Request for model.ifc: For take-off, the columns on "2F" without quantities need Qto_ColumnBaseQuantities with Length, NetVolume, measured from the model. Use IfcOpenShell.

First a look at what the model holds.

```python
import ifcopenshell
import ifcopenshell.util.element
import ifcopenshell.util.unit

model = ifcopenshell.open("model.ifc")
print(model.schema)
for unit_type in ("LENGTHUNIT", "AREAUNIT", "VOLUMEUNIT"):
    print(unit_type, ifcopenshell.util.unit.calculate_unit_scale(model, unit_type))
storey = next(s for s in model.by_type("IfcBuildingStorey") if s.Name == "2F")
columns = [e for e in ifcopenshell.util.element.get_decomposition(storey) if e.is_a("IfcColumn")]
for e in sorted(columns, key=lambda e: e.id()):
    print(e.id(), e.is_a(), e.Name, list(ifcopenshell.util.element.get_psets(e, qtos_only=True)), sep=" | ")
```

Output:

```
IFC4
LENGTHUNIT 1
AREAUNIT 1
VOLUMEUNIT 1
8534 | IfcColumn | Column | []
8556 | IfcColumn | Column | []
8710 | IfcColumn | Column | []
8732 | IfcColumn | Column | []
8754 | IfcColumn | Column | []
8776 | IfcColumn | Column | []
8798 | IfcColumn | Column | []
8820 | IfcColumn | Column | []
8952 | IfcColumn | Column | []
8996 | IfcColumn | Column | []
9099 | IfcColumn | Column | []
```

```python
import ifcopenshell
import ifcopenshell.api.pset
import ifcopenshell.geom
import ifcopenshell.util.element
import ifcopenshell.util.shape
import ifcopenshell.util.unit

model = ifcopenshell.open("model.ifc")
unit_scale = ifcopenshell.util.unit.calculate_unit_scale(model)
volume_scale = ifcopenshell.util.unit.calculate_unit_scale(model, "VOLUMEUNIT")
settings = ifcopenshell.geom.settings()

storey = next(s for s in model.by_type("IfcBuildingStorey") if s.Name == "2F")
columns = [e for e in ifcopenshell.util.element.get_decomposition(storey) if e.is_a("IfcColumn")]

for e in sorted(columns, key=lambda e: e.id()):
    if ifcopenshell.util.element.get_psets(e, qtos_only=True, should_inherit=False):
        continue
    # Geometry comes back in metres, in the element's own axes.
    shape = ifcopenshell.geom.create_shape(settings, e)
    values = {
        "Length": ifcopenshell.util.shape.get_z(shape.geometry) / unit_scale,
        "NetVolume": ifcopenshell.util.shape.get_volume(shape.geometry) / volume_scale,
    }
    qto = ifcopenshell.api.pset.add_qto(model, product=e, name="Qto_ColumnBaseQuantities")
    ifcopenshell.api.pset.edit_qto(model, qto=qto, properties=values)
    print(e.id(), {k: round(v, 3) for k, v in values.items()})

model.write("model_edited.ifc")
```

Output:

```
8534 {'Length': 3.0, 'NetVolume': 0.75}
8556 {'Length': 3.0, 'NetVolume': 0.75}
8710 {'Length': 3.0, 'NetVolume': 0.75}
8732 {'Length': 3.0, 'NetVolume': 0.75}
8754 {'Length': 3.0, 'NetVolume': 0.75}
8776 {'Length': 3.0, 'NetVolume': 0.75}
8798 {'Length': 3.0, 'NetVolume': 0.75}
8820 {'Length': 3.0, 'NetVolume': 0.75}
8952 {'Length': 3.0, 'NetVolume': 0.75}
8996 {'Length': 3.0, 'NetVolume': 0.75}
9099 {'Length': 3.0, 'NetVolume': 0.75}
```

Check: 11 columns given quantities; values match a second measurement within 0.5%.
